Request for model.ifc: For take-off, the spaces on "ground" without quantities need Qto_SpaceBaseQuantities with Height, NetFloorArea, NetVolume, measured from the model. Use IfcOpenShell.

First a look at what the model holds.

```python
import ifcopenshell
import ifcopenshell.util.element
import ifcopenshell.util.unit

model = ifcopenshell.open("model.ifc")
print(model.schema)
for unit_type in ("LENGTHUNIT", "AREAUNIT", "VOLUMEUNIT"):
    print(unit_type, ifcopenshell.util.unit.calculate_unit_scale(model, unit_type))
storey = next(s for s in model.by_type("IfcBuildingStorey") if s.Name == "ground")
spaces = [e for e in ifcopenshell.util.element.get_decomposition(storey) if e.is_a("IfcSpace")]
for e in sorted(spaces, key=lambda e: e.id()):
    print(e.id(), e.is_a(), e.Name, list(ifcopenshell.util.element.get_psets(e, qtos_only=True)), sep=" | ")
```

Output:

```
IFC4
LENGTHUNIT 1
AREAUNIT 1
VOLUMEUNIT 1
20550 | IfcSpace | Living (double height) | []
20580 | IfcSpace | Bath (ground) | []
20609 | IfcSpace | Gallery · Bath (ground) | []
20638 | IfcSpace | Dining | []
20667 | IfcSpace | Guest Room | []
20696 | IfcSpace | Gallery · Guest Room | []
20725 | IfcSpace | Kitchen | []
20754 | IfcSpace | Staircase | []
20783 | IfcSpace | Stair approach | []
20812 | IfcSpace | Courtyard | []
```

```python
import ifcopenshell
import ifcopenshell.api.pset
import ifcopenshell.geom
import ifcopenshell.util.element
import ifcopenshell.util.shape
import ifcopenshell.util.unit

model = ifcopenshell.open("model.ifc")
unit_scale = ifcopenshell.util.unit.calculate_unit_scale(model)
area_scale = ifcopenshell.util.unit.calculate_unit_scale(model, "AREAUNIT")
volume_scale = ifcopenshell.util.unit.calculate_unit_scale(model, "VOLUMEUNIT")
settings = ifcopenshell.geom.settings()

storey = next(s for s in model.by_type("IfcBuildingStorey") if s.Name == "ground")
spaces = [e for e in ifcopenshell.util.element.get_decomposition(storey) if e.is_a("IfcSpace")]

for e in sorted(spaces, key=lambda e: e.id()):
    if ifcopenshell.util.element.get_psets(e, qtos_only=True, should_inherit=False):
        continue
    # Geometry comes back in metres, in the element's own axes.
    shape = ifcopenshell.geom.create_shape(settings, e)
    values = {
        "Height": ifcopenshell.util.shape.get_z(shape.geometry) / unit_scale,
        "NetFloorArea": ifcopenshell.util.shape.get_footprint_area(shape.geometry) / area_scale,
        "NetVolume": ifcopenshell.util.shape.get_volume(shape.geometry) / volume_scale,
    }
    qto = ifcopenshell.api.pset.add_qto(model, product=e, name="Qto_SpaceBaseQuantities")
    ifcopenshell.api.pset.edit_qto(model, qto=qto, properties=values)
    print(e.id(), {k: round(v, 3) for k, v in values.items()})

model.write("model_edited.ifc")
```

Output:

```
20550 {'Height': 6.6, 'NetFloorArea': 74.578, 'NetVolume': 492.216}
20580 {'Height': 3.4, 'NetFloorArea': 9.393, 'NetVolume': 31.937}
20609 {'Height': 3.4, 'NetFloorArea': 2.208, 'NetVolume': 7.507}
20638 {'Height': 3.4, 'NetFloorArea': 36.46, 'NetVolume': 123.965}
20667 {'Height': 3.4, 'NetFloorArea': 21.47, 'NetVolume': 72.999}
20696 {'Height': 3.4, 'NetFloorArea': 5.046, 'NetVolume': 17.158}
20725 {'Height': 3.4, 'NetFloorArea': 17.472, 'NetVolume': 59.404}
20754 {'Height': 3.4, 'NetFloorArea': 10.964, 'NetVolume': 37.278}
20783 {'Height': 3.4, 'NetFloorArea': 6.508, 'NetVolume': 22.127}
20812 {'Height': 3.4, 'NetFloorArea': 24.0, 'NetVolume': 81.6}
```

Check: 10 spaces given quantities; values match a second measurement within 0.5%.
